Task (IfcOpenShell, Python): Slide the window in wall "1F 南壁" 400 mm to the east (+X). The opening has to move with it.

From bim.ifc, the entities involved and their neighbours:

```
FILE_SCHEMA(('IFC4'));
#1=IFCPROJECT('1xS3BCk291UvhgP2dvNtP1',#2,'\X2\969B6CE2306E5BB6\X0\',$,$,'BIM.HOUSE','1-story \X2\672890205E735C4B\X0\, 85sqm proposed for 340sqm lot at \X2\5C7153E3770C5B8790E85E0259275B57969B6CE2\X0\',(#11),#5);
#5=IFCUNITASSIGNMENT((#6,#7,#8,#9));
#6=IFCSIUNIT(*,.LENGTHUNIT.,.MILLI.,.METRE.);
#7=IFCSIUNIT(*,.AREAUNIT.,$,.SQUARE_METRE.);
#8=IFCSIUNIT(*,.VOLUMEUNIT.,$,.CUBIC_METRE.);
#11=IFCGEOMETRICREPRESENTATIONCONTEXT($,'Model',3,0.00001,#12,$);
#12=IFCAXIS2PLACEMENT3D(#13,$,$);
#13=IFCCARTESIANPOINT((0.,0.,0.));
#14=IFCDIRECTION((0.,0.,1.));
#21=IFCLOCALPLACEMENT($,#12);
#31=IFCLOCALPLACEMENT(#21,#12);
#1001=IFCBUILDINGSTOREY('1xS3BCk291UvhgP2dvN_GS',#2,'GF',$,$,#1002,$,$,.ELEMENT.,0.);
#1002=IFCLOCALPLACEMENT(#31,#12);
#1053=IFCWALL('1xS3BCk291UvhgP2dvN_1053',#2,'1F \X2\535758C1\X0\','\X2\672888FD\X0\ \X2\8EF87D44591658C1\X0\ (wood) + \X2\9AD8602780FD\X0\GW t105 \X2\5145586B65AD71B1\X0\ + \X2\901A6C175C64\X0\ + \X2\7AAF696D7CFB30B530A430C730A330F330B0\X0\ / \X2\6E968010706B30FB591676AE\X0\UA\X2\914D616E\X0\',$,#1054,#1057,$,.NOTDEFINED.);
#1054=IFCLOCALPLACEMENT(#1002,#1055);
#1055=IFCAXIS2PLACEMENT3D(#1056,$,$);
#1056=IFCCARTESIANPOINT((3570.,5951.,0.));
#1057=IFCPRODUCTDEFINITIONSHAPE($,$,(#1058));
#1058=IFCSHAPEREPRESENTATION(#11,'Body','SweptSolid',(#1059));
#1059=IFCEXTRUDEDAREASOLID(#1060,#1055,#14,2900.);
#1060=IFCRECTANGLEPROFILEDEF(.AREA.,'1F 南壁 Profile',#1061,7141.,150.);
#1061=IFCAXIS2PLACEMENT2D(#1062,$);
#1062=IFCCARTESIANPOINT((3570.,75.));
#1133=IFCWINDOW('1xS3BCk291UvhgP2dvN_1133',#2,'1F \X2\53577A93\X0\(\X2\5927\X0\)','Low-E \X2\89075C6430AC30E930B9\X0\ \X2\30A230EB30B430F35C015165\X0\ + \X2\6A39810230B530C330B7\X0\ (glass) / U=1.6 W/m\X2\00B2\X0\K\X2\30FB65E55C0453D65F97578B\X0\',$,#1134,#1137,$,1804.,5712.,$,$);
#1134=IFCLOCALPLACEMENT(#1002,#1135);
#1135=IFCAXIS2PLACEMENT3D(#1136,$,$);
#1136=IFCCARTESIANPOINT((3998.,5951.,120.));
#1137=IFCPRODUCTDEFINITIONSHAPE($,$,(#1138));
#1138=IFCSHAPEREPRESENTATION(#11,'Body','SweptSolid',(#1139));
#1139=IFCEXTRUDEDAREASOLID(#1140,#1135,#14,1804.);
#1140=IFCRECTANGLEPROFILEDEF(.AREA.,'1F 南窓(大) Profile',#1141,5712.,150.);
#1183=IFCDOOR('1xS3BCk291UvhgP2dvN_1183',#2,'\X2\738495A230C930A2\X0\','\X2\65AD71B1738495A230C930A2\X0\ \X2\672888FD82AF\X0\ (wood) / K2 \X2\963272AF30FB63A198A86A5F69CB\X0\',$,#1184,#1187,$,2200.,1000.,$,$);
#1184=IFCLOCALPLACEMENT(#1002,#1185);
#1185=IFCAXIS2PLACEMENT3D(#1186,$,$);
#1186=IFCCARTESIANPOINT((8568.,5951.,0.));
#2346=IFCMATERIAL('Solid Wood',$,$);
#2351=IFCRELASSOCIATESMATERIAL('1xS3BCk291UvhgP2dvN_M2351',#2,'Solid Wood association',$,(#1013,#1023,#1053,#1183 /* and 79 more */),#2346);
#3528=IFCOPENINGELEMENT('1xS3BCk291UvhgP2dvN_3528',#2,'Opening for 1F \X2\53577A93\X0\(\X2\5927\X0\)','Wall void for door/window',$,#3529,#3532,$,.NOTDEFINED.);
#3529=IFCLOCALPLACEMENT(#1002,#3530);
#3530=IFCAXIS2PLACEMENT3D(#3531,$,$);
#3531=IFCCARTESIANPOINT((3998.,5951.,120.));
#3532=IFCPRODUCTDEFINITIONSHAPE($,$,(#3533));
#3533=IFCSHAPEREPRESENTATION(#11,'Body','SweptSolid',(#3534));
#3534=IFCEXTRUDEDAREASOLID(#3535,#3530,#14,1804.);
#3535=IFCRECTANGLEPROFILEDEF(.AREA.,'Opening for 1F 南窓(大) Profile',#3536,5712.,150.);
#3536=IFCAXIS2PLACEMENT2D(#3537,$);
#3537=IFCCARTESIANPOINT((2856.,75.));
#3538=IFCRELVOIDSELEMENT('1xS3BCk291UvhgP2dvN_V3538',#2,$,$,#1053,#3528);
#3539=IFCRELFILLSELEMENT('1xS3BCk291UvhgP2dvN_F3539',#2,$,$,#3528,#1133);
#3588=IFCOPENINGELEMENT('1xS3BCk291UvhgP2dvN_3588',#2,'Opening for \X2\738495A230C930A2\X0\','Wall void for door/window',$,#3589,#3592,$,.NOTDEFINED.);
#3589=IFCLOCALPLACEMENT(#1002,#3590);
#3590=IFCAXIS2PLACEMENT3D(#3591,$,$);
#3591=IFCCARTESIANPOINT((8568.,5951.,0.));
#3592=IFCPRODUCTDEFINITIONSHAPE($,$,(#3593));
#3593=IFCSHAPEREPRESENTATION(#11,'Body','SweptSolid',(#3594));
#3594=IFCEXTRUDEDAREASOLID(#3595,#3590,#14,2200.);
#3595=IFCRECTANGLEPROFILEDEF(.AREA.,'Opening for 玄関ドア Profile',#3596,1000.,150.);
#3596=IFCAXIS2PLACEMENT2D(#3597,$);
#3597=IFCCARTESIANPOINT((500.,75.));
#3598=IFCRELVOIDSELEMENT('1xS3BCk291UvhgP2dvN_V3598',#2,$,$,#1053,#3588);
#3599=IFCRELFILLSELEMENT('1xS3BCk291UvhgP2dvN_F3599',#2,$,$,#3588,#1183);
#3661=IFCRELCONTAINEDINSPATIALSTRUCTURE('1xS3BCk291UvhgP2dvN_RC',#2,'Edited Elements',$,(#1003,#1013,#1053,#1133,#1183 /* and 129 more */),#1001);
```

```python
import ifcopenshell
import ifcopenshell.api.geometry
import ifcopenshell.util.placement

model = ifcopenshell.open("bim.ifc")

window = model.by_guid("1xS3BCk291UvhgP2dvN_1133")
opening = window.FillsVoids[0].RelatingOpeningElement
wall = opening.VoidsElements[0].RelatingBuildingElement

wall_matrix = ifcopenshell.util.placement.get_local_placement(wall.ObjectPlacement)
shift = wall_matrix[:3, 0] * 400.0
before = ifcopenshell.util.placement.get_local_placement(window.ObjectPlacement)[:3, 3].copy()

# The window is not placed relative to its opening, so move both.
for product in (opening, window):
    matrix = ifcopenshell.util.placement.get_local_placement(product.ObjectPlacement)
    matrix[:3, 3] += shift
    ifcopenshell.api.geometry.edit_object_placement(model, product=product, matrix=matrix, is_si=False)

after = ifcopenshell.util.placement.get_local_placement(window.ObjectPlacement)[:3, 3]
print("window moved by", (after - before).round(3) + 0.0)

model.write("bim-out.ifc")
```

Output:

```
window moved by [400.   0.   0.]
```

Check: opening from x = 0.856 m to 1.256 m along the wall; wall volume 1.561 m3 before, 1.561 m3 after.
